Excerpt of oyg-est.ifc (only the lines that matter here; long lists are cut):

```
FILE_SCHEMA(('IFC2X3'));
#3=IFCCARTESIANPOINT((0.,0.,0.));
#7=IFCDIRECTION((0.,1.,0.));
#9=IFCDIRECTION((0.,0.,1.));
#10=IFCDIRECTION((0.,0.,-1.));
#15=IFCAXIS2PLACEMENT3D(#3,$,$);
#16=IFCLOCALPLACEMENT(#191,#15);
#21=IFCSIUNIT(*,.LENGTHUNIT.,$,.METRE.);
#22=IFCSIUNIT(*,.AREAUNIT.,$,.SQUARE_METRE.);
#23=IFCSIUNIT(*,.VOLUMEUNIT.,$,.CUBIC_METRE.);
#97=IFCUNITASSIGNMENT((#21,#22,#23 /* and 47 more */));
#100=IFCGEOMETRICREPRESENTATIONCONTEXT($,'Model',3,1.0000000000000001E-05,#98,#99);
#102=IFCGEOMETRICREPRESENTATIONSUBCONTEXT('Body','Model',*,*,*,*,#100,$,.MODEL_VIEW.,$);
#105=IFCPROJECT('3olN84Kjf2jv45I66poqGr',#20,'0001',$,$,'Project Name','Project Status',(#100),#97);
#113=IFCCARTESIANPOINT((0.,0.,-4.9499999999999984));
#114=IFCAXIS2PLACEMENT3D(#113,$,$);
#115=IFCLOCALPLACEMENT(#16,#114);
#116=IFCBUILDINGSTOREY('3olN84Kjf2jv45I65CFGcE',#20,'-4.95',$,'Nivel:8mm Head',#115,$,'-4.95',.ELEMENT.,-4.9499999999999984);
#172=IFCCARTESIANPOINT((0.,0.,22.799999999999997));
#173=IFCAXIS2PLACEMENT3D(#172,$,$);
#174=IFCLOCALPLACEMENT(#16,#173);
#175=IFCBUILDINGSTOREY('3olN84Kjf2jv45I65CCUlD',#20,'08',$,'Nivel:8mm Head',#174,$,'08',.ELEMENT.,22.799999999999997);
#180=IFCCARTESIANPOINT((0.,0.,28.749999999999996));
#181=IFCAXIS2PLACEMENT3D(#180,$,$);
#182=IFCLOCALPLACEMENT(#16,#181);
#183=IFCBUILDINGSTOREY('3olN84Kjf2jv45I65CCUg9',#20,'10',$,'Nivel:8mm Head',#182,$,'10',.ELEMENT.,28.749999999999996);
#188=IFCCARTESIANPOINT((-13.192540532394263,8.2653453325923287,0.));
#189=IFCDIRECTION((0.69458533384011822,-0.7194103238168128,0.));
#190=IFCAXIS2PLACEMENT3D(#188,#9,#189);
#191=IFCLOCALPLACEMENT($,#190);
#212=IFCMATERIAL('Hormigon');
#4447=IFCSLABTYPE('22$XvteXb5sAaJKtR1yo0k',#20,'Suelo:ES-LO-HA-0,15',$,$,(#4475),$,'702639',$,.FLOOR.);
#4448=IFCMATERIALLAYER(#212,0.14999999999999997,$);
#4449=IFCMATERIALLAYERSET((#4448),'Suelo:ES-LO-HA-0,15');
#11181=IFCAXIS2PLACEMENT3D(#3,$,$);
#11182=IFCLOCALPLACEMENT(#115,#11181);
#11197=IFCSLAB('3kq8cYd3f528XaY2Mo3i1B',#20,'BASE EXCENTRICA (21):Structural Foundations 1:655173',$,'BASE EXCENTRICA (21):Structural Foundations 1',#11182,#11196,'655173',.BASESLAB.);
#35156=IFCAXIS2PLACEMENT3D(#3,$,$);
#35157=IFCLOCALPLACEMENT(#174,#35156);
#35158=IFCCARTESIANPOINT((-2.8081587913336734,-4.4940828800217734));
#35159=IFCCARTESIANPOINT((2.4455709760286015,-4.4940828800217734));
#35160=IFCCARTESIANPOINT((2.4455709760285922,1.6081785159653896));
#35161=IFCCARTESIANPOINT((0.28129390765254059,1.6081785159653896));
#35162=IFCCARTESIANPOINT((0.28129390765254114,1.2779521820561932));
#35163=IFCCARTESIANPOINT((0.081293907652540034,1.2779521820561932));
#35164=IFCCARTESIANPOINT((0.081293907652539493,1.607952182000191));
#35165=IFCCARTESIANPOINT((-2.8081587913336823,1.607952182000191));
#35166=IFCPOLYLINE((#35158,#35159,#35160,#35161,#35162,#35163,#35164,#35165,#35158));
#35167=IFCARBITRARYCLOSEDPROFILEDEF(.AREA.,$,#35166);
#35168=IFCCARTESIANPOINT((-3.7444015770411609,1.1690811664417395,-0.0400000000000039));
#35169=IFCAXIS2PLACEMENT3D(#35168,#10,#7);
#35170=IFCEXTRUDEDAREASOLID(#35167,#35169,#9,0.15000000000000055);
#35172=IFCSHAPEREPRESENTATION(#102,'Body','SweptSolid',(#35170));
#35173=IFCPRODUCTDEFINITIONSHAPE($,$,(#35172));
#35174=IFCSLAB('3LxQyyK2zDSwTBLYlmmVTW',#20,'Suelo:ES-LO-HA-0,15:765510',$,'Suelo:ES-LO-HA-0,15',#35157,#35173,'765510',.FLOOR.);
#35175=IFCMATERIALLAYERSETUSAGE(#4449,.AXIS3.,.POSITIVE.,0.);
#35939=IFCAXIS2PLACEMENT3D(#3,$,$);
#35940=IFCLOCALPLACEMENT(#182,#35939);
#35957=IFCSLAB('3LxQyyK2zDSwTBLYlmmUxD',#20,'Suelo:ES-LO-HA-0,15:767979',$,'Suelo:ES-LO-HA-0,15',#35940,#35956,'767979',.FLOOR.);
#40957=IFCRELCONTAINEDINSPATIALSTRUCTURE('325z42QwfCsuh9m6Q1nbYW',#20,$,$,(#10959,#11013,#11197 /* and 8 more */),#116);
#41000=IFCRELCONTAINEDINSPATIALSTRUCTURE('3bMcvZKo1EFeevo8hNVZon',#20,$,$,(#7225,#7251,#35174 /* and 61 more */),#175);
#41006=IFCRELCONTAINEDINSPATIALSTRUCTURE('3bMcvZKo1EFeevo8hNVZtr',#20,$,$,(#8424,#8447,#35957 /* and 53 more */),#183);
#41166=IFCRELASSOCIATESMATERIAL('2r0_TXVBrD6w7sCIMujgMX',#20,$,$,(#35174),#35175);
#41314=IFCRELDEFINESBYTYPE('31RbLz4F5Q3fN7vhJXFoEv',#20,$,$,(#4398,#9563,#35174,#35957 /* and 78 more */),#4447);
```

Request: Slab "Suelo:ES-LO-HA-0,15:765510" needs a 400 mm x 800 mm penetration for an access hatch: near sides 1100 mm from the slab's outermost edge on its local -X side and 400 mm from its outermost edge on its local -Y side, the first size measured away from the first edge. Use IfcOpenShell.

```python
import numpy as np
import ifcopenshell
import ifcopenshell.api.feature
import ifcopenshell.api.geometry
import ifcopenshell.api.root
import ifcopenshell.geom
import ifcopenshell.util.placement
import ifcopenshell.util.representation
import ifcopenshell.util.shape
import ifcopenshell.util.unit

model = ifcopenshell.open("oyg-est.ifc")
unit_scale = ifcopenshell.util.unit.calculate_unit_scale(model)
settings = ifcopenshell.geom.settings()


def volume(element):
    """Net volume in cubic metres, openings subtracted."""
    shape = ifcopenshell.geom.create_shape(settings, element)
    return ifcopenshell.util.shape.get_volume(shape.geometry)


slab = model.by_guid("3LxQyyK2zDSwTBLYlmmVTW")
before = volume(slab)

# Extent in the slab's own axes, in metres. The edges named are its -X and -Y sides.
slab_shape = ifcopenshell.geom.create_shape(settings, slab)
vertices = ifcopenshell.util.shape.get_vertices(slab_shape.geometry)
x_min, y_min, bottom = vertices.min(axis=0)
top = vertices[:, 2].max()

opening = ifcopenshell.api.root.create_entity(model, ifc_class="IfcOpeningElement", name="Access hatch opening")
context = ifcopenshell.util.representation.get_context(model, "Model", "Body", "MODEL_VIEW")
width, depth = 0.4, 0.8
outline = [(0.0, 0.0), (width, 0.0), (width, depth), (0.0, depth), (0.0, 0.0)]
# Overshoot both faces by 50 mm so the cut is clean.
shape = ifcopenshell.api.geometry.add_slab_representation(
    model, context=context, depth=top - bottom + 0.1, polyline=outline
)
ifcopenshell.api.geometry.assign_representation(model, product=opening, representation=shape)

matrix = ifcopenshell.util.placement.get_local_placement(slab.ObjectPlacement)
matrix[:, 3] = matrix @ np.append(np.array([x_min + 1.1, y_min + 0.4, bottom - 0.05]) / unit_scale, 1.0)
ifcopenshell.api.geometry.edit_object_placement(model, product=opening, matrix=matrix, is_si=False)
ifcopenshell.api.feature.add_feature(model, feature=opening, element=slab)

after = volume(slab)

print(f"slab volume {before:.3f} -> {after:.3f} m3")

model.write("oyg-est_rev.ifc")
```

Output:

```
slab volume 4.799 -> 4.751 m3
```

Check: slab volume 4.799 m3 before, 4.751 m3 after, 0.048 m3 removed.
